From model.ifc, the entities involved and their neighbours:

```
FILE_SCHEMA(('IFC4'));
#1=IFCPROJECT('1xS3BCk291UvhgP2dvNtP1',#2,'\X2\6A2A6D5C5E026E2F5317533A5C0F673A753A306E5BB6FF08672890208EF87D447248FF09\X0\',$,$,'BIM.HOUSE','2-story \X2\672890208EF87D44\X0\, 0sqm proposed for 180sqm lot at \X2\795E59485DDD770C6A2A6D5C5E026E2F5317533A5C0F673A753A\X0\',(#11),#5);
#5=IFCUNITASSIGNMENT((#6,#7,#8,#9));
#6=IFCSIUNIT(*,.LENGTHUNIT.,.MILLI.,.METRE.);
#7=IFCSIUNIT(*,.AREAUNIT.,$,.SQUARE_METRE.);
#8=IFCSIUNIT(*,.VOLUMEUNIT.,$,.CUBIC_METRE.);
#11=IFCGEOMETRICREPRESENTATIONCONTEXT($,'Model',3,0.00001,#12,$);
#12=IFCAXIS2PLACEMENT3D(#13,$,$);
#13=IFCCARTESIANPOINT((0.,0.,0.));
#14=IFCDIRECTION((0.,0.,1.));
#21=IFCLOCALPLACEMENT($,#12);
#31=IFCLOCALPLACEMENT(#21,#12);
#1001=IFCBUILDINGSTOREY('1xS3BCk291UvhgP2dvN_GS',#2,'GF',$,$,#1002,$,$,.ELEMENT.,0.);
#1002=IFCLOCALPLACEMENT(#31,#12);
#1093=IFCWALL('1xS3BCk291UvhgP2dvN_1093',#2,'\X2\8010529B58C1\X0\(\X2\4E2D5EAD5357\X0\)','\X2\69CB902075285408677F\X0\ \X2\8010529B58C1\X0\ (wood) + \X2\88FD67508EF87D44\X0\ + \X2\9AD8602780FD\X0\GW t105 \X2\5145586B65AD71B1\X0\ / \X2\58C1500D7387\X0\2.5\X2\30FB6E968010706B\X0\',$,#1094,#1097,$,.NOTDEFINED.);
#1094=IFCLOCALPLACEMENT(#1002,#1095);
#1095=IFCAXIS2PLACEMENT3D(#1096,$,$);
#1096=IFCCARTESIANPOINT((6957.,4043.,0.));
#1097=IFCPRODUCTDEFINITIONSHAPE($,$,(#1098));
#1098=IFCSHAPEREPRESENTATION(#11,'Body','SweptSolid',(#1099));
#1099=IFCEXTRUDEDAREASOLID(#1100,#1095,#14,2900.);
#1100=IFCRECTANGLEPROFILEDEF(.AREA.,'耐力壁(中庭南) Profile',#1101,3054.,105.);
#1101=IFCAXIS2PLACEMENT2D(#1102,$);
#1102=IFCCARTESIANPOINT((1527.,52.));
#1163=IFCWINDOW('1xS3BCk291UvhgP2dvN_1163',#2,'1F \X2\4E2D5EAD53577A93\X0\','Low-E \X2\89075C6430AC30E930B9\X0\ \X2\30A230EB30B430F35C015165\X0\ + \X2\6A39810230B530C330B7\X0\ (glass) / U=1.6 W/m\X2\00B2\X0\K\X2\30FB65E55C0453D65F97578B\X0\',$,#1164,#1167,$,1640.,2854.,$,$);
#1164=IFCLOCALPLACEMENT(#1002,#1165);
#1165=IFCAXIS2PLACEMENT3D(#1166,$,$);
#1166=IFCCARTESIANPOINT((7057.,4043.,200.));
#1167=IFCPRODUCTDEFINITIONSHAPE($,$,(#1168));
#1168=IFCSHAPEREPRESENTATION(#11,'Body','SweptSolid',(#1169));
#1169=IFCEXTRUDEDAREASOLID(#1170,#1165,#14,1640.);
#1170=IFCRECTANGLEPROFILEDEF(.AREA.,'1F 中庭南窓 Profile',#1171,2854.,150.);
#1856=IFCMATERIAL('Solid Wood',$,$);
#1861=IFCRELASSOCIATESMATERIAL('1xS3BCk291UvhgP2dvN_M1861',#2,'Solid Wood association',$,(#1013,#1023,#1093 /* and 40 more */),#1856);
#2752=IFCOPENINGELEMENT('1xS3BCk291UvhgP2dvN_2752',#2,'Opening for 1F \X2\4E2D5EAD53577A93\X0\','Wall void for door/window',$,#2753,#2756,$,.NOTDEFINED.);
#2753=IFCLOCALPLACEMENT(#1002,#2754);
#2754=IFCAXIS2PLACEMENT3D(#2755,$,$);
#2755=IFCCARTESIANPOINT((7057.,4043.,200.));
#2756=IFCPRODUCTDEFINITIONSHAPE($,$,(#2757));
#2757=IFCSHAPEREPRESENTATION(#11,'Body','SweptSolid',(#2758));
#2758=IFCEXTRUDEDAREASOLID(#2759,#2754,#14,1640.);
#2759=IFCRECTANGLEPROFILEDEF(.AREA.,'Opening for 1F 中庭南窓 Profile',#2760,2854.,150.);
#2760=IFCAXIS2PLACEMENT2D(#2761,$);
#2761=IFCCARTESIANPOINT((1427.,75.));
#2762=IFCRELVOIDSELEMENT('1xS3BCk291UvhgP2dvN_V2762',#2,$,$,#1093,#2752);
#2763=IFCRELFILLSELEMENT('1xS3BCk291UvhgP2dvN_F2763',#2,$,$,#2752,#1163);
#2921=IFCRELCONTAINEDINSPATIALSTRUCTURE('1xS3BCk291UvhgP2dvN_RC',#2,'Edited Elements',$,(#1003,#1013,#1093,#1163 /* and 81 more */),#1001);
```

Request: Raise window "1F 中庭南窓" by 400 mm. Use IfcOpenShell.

```python
import numpy as np
import ifcopenshell
import ifcopenshell.api.geometry
import ifcopenshell.util.placement
import ifcopenshell.util.unit

model = ifcopenshell.open("model.ifc")
unit_scale = ifcopenshell.util.unit.calculate_unit_scale(model)

window = model.by_id(1163)
opening = window.FillsVoids[0].RelatingOpeningElement
dz = 0.4 / unit_scale

shift = np.array([0.0, 0.0, dz])
# The window is not placed relative to its opening, so move both.
for product in (opening, window):
    matrix = ifcopenshell.util.placement.get_local_placement(product.ObjectPlacement)
    matrix[:3, 3] += shift
    ifcopenshell.api.geometry.edit_object_placement(model, product=product, matrix=matrix, is_si=False)

print(f"moved by {dz * unit_scale:+.3f} m")

model.write("model_updated.ifc")
```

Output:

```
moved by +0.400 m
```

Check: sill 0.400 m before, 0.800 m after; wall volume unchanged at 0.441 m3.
